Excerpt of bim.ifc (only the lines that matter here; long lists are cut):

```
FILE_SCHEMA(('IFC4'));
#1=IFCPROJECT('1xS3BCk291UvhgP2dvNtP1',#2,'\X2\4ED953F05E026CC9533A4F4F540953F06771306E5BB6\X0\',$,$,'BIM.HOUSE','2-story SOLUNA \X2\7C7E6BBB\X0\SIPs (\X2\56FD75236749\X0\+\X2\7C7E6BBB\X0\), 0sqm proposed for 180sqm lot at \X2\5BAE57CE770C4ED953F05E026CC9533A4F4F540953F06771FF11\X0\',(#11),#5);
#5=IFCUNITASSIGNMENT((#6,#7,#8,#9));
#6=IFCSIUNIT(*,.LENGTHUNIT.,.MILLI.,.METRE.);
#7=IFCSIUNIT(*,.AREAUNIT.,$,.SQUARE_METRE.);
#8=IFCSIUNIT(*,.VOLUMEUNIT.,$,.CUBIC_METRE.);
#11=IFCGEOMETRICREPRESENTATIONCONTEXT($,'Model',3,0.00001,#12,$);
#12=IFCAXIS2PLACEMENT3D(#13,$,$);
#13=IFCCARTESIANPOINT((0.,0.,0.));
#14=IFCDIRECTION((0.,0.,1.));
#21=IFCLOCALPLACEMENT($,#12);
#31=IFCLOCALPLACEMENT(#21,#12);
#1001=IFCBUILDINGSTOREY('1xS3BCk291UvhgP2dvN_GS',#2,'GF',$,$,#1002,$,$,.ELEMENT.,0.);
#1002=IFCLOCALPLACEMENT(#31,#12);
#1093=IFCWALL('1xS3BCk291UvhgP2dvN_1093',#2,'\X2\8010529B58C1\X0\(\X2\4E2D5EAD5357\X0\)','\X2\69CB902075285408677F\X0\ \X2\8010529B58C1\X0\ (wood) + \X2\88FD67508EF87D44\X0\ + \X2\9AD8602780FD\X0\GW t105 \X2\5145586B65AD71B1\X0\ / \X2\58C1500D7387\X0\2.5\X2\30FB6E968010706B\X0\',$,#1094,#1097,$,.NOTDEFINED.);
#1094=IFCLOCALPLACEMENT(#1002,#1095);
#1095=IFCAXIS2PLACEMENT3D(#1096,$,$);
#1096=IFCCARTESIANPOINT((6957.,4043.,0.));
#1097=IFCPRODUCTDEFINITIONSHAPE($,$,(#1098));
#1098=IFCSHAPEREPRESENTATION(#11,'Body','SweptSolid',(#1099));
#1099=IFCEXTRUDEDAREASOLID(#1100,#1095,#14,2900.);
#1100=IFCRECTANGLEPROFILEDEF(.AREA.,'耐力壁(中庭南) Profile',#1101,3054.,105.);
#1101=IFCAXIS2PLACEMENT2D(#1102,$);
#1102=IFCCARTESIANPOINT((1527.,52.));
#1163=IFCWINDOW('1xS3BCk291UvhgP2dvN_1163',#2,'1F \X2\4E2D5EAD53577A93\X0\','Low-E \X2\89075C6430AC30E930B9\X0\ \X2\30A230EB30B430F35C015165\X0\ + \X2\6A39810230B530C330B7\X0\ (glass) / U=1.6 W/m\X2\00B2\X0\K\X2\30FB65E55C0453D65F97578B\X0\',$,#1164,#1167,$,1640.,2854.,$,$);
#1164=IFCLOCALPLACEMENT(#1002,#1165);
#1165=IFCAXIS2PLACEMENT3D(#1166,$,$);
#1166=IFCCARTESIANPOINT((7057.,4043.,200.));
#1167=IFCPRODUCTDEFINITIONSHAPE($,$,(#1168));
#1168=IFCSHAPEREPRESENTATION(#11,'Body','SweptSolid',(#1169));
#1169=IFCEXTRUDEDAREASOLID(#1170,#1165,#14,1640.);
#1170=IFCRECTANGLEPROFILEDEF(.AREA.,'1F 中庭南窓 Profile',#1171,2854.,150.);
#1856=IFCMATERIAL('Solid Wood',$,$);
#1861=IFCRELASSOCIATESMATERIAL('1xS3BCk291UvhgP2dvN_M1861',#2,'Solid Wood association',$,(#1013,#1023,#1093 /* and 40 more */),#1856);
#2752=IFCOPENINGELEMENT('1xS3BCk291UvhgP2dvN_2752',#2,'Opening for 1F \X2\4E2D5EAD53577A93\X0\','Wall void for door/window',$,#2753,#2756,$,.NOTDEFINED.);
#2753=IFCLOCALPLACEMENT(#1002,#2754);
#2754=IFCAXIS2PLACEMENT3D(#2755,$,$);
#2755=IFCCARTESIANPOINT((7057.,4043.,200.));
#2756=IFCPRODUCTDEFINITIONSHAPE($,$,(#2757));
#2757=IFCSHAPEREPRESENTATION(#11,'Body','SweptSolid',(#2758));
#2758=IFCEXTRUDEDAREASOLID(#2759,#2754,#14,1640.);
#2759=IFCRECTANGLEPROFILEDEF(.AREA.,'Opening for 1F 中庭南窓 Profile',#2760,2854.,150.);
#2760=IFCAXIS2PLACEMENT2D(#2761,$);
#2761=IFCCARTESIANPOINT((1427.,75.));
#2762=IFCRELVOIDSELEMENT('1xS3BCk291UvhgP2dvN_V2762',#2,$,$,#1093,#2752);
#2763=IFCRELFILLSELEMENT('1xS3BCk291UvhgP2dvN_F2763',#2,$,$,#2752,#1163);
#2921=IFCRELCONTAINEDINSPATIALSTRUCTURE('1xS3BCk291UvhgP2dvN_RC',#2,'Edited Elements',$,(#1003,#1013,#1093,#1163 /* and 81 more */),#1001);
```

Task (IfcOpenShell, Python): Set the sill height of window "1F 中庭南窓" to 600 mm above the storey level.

```python
import numpy as np
import ifcopenshell
import ifcopenshell.api.geometry
import ifcopenshell.geom
import ifcopenshell.util.element
import ifcopenshell.util.placement
import ifcopenshell.util.shape
import ifcopenshell.util.unit

model = ifcopenshell.open("bim.ifc")
unit_scale = ifcopenshell.util.unit.calculate_unit_scale(model)

window = model.by_guid("1xS3BCk291UvhgP2dvN_1163")
opening = window.FillsVoids[0].RelatingOpeningElement
storey = ifcopenshell.util.element.get_container(window, ifc_class="IfcBuildingStorey")
level = ifcopenshell.util.placement.get_local_placement(storey.ObjectPlacement)[2, 3]

# The opening's origin need not be at the sill, so measure its lowest point.
shape = ifcopenshell.geom.create_shape(ifcopenshell.geom.settings(), opening)
bottom = ifcopenshell.util.shape.get_shape_bottom_elevation(shape, shape.geometry) / unit_scale
dz = level + 0.6 / unit_scale - bottom

shift = np.array([0.0, 0.0, dz])
# The window is not placed relative to its opening, so move both.
for product in (opening, window):
    matrix = ifcopenshell.util.placement.get_local_placement(product.ObjectPlacement)
    matrix[:3, 3] += shift
    ifcopenshell.api.geometry.edit_object_placement(model, product=product, matrix=matrix, is_si=False)

print(f"moved by {dz * unit_scale:+.3f} m")

model.write("bim_rev.ifc")
```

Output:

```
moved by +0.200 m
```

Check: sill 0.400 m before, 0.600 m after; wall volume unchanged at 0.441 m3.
